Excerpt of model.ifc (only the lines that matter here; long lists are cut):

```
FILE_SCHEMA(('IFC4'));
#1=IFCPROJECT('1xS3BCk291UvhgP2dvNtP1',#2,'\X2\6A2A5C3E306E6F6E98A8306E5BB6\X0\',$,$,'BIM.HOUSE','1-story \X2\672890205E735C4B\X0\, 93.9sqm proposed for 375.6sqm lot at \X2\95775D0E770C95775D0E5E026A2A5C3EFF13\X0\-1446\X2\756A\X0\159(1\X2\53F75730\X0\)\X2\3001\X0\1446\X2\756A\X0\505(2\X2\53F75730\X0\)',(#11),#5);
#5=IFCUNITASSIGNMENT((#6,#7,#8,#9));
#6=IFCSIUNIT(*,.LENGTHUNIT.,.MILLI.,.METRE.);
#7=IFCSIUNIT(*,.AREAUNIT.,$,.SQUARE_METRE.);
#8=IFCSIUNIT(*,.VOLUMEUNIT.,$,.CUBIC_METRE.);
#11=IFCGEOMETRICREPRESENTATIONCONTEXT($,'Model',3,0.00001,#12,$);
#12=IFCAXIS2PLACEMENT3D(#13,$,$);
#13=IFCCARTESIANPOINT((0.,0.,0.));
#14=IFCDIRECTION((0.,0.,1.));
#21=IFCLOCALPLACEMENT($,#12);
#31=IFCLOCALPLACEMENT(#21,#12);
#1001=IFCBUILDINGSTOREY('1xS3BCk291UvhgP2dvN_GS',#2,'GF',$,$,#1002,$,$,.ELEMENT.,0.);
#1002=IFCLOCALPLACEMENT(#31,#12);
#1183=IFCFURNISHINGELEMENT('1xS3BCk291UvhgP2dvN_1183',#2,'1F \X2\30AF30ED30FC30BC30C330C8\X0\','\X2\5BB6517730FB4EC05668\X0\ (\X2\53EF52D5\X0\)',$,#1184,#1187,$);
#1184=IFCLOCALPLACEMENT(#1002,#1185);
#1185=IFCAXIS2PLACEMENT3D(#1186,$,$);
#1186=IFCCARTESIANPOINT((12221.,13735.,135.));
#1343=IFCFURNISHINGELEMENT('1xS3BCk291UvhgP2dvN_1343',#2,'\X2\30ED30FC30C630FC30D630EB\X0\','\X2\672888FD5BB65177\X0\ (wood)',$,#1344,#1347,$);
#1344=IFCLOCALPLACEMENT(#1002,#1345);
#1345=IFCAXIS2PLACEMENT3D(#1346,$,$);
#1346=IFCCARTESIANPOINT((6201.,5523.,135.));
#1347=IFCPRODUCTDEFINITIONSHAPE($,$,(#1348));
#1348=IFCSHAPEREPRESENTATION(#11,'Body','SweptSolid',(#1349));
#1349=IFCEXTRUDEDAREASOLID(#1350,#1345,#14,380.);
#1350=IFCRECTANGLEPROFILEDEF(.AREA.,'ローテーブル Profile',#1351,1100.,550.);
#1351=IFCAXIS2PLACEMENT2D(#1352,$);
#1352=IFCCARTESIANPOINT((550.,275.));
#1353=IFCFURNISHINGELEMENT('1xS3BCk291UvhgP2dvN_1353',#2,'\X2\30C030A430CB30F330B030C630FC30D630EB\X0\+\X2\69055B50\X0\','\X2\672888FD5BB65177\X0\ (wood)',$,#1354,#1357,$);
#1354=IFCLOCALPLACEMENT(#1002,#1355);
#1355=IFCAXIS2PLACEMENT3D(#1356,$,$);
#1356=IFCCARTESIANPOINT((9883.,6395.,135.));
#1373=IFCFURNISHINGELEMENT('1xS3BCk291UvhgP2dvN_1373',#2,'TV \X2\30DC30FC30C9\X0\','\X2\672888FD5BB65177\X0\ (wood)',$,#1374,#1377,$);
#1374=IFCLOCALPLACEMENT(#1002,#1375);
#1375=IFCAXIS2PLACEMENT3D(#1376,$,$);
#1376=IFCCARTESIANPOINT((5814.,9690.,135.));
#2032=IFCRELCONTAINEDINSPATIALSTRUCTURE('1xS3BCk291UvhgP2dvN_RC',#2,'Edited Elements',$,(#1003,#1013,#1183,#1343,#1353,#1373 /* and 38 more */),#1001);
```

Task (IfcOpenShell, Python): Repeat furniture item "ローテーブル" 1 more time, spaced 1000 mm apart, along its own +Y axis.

```python
import ifcopenshell
import ifcopenshell.api.geometry
import ifcopenshell.api.root
import ifcopenshell.util.element
import ifcopenshell.util.placement
import ifcopenshell.util.unit

model = ifcopenshell.open("model.ifc")
unit_scale = ifcopenshell.util.unit.calculate_unit_scale(model)


def reuse_history(source, copy):
    """copy_class also copies each property set's owner history, people and application; keep the originals."""
    for rel in copy.IsDefinedBy:
        if rel.is_a("IfcRelDefinesByProperties") and (history := rel.RelatingPropertyDefinition.OwnerHistory):
            rel.RelatingPropertyDefinition.OwnerHistory = source.OwnerHistory
            ifcopenshell.util.element.remove_deep2(model, history)


source = model.by_id(1343)
base = ifcopenshell.util.placement.get_local_placement(source.ObjectPlacement)
step = base[:3, 1] * 1 / unit_scale

for i in range(1, 2):
    copy = ifcopenshell.api.root.copy_class(model, product=source)
    copy.Representation = ifcopenshell.util.element.copy_deep(
        model, source.Representation, exclude=["IfcGeometricRepresentationContext", "IfcRepresentationMap"]
    )
    reuse_history(source, copy)
    matrix = base.copy()
    matrix[:3, 3] += i * step
    print("added at", matrix[:3, 3].round(3) + 0.0)
    ifcopenshell.api.geometry.edit_object_placement(model, product=copy, matrix=matrix, is_si=False)

model.write("model_updated.ifc")
```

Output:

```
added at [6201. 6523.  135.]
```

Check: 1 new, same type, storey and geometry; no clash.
